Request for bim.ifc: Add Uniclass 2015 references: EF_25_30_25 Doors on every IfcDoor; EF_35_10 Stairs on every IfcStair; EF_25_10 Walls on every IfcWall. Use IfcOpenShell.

First a look at what the model holds.

```python
import ifcopenshell

model = ifcopenshell.open("bim.ifc")
print(model.schema)
print("classifications:", [c.Name for c in model.by_type("IfcClassification")])
for ifc_class in ("IfcDoor", "IfcRoof", "IfcStair", "IfcWall", "IfcWindow"):
    print(ifc_class, len(model.by_type(ifc_class)))
```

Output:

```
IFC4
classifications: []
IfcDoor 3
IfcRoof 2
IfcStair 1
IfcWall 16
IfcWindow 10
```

```python
import ifcopenshell
import ifcopenshell.api.classification

model = ifcopenshell.open("bim.ifc")

system = ifcopenshell.api.classification.add_classification(model, classification="Uniclass 2015")

codes = {
    "IfcDoor": ("EF_25_30_25", "Doors"),
    "IfcStair": ("EF_35_10", "Stairs"),
    "IfcWall": ("EF_25_10", "Walls"),
}
for ifc_class, (code, name) in codes.items():
    products = model.by_type(ifc_class)
    ifcopenshell.api.classification.add_reference(
        model, products=products, classification=system, identification=code, name=name
    )
    print(code, len(products))

model.write("bim_rev.ifc")
```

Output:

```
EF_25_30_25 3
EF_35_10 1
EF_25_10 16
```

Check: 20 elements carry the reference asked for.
